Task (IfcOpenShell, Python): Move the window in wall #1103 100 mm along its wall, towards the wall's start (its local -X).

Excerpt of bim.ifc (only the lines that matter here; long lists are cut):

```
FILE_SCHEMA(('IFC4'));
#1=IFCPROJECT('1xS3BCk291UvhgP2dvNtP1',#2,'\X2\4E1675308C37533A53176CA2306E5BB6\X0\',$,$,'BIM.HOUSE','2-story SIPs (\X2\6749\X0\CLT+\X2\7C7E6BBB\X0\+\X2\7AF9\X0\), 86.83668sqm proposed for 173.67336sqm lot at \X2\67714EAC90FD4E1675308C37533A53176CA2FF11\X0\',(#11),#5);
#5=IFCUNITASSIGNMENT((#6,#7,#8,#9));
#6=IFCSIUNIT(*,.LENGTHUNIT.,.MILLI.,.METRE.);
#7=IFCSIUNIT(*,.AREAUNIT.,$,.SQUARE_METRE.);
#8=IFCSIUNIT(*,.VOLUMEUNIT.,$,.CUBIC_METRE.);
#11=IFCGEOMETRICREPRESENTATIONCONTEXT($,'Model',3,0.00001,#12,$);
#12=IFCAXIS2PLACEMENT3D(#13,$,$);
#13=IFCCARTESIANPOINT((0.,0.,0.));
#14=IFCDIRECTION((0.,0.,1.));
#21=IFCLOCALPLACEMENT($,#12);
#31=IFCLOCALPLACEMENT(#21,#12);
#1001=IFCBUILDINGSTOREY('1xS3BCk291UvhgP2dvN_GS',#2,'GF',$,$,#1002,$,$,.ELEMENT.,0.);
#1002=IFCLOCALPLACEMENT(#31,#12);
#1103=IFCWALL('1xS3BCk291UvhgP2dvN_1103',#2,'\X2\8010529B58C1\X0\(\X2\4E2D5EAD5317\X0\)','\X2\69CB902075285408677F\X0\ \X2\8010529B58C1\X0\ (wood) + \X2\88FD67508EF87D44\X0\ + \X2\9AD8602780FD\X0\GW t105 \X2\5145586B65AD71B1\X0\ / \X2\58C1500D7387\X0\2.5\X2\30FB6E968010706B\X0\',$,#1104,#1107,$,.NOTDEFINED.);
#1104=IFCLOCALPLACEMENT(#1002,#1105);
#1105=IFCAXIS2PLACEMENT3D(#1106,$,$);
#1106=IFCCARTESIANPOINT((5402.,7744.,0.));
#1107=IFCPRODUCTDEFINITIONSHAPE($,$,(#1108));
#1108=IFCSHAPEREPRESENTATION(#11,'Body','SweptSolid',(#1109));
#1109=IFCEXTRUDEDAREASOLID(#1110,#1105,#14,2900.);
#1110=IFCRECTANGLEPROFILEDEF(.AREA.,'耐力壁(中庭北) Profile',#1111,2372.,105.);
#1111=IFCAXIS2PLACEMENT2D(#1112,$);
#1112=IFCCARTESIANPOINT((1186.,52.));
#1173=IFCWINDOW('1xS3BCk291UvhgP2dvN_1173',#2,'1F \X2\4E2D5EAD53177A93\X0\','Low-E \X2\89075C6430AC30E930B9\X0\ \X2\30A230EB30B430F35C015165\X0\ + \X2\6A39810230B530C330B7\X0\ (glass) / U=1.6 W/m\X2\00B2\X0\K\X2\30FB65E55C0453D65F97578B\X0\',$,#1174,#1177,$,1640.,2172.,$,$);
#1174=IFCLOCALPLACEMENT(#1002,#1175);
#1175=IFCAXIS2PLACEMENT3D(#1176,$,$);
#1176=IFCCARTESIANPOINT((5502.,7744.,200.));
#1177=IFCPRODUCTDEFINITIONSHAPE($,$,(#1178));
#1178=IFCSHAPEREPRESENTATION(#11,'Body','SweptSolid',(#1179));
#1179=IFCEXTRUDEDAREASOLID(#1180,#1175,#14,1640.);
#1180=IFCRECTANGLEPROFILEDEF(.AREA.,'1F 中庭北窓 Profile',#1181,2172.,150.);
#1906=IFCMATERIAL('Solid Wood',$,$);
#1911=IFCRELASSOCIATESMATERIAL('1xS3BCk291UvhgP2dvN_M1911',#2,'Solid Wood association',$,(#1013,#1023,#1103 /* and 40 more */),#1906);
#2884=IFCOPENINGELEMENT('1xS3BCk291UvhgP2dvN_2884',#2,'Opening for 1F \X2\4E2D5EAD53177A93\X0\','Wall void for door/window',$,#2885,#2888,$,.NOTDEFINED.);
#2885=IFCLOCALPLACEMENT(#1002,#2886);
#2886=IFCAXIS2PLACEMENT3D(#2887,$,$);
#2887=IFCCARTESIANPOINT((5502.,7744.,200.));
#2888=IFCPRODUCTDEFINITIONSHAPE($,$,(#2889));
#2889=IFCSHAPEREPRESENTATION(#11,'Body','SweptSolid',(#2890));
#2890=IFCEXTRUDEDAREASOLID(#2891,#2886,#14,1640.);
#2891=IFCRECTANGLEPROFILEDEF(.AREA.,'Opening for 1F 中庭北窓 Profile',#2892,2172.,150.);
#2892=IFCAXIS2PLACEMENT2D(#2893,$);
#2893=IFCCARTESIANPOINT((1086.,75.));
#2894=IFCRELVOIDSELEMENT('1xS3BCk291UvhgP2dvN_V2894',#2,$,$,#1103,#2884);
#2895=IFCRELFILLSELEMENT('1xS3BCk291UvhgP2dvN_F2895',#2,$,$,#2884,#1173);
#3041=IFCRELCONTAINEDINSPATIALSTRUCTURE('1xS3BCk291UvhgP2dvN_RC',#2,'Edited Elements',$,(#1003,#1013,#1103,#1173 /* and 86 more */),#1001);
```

```python
import ifcopenshell
import ifcopenshell.api.geometry
import ifcopenshell.util.placement
import ifcopenshell.util.unit

model = ifcopenshell.open("bim.ifc")
unit_scale = ifcopenshell.util.unit.calculate_unit_scale(model)

window = model.by_id(1173)
opening = window.FillsVoids[0].RelatingOpeningElement
wall = opening.VoidsElements[0].RelatingBuildingElement

wall_matrix = ifcopenshell.util.placement.get_local_placement(wall.ObjectPlacement)
shift = wall_matrix[:3, 0] * -0.1 / unit_scale
before = ifcopenshell.util.placement.get_local_placement(window.ObjectPlacement)[:3, 3].copy()

# The window is not placed relative to its opening, so move both.
for product in (opening, window):
    matrix = ifcopenshell.util.placement.get_local_placement(product.ObjectPlacement)
    matrix[:3, 3] += shift
    ifcopenshell.api.geometry.edit_object_placement(model, product=product, matrix=matrix, is_si=False)

after = ifcopenshell.util.placement.get_local_placement(window.ObjectPlacement)[:3, 3]
print("window moved by", (after - before).round(3) + 0.0)

model.write("bim_edited.ifc")
```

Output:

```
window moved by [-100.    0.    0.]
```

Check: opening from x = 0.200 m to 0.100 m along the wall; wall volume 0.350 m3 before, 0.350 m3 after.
